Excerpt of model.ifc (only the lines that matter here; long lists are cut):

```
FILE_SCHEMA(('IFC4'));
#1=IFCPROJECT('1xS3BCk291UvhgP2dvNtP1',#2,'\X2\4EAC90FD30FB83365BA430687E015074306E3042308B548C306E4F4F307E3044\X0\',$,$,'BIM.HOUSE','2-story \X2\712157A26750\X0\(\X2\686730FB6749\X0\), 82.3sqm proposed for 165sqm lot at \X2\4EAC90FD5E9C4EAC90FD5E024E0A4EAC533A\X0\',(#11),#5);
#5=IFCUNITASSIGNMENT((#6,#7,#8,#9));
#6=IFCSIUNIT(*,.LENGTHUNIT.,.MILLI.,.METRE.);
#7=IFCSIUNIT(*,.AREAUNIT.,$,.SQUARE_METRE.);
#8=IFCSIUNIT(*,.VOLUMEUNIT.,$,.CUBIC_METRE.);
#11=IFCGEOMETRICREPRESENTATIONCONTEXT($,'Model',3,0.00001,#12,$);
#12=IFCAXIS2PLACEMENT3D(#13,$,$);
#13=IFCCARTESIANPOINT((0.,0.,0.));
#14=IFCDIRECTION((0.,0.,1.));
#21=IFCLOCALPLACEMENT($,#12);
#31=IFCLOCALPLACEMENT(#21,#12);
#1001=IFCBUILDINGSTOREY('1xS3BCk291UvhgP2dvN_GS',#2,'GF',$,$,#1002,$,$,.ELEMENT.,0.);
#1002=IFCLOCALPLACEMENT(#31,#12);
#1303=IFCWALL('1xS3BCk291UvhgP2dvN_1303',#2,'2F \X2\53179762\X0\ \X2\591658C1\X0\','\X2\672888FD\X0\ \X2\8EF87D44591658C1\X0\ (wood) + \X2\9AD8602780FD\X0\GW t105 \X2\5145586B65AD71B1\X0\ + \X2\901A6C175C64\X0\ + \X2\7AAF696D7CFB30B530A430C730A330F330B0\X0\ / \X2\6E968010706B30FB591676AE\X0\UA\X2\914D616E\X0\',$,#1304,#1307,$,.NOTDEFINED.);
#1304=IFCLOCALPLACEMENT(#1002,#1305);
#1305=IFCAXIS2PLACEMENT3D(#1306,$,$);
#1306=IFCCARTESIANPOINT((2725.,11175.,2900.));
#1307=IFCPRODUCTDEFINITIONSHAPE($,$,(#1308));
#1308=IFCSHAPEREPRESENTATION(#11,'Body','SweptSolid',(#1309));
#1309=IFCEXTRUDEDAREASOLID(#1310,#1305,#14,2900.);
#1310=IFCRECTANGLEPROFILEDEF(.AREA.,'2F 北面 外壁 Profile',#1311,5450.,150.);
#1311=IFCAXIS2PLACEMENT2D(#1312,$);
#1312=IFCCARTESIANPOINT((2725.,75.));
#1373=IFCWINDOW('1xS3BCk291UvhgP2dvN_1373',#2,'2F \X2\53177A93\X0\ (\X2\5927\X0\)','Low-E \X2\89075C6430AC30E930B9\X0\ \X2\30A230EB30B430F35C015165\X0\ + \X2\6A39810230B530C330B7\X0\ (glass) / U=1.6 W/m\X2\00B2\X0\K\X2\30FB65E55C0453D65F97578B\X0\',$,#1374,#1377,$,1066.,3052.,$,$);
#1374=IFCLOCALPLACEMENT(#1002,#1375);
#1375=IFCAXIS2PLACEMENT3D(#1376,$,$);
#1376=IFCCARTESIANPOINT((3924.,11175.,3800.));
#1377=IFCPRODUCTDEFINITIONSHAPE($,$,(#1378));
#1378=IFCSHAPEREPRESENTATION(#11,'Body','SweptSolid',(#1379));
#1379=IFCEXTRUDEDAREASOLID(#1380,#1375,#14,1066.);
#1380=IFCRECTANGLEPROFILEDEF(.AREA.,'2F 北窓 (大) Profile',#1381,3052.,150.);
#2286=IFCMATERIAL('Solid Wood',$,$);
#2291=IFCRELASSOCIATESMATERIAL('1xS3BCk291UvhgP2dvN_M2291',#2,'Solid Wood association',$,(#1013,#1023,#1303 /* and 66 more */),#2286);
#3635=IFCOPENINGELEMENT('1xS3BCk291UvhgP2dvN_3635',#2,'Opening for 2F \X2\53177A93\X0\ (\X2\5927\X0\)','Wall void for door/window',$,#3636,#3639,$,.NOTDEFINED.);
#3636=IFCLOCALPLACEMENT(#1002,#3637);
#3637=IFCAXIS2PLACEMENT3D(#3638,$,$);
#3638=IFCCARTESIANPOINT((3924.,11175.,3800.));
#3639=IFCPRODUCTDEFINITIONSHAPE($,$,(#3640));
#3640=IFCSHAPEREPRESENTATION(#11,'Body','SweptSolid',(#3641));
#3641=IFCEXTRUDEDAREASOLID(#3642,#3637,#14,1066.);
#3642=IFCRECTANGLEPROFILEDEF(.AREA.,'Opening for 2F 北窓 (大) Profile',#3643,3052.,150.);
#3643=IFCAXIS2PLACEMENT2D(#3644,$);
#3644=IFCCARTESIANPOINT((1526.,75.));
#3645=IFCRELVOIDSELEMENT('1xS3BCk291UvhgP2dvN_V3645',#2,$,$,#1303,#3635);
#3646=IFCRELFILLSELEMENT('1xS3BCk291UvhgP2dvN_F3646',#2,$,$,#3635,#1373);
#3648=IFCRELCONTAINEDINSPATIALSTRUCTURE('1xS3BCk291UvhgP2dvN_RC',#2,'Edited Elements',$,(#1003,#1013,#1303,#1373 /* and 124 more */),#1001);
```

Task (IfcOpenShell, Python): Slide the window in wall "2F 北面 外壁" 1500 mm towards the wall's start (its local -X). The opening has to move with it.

```python
import ifcopenshell
import ifcopenshell.api.geometry
import ifcopenshell.util.placement
import ifcopenshell.util.unit

model = ifcopenshell.open("model.ifc")
unit_scale = ifcopenshell.util.unit.calculate_unit_scale(model)

window = model.by_id(1373)
opening = window.FillsVoids[0].RelatingOpeningElement
wall = opening.VoidsElements[0].RelatingBuildingElement

wall_matrix = ifcopenshell.util.placement.get_local_placement(wall.ObjectPlacement)
shift = wall_matrix[:3, 0] * -1.5 / unit_scale
before = ifcopenshell.util.placement.get_local_placement(window.ObjectPlacement)[:3, 3].copy()

# The window is not placed relative to its opening, so move both.
for product in (opening, window):
    matrix = ifcopenshell.util.placement.get_local_placement(product.ObjectPlacement)
    matrix[:3, 3] += shift
    ifcopenshell.api.geometry.edit_object_placement(model, product=product, matrix=matrix, is_si=False)

after = ifcopenshell.util.placement.get_local_placement(window.ObjectPlacement)[:3, 3]
print("window moved by", (after - before).round(3) + 0.0)

model.write("model_rev.ifc")
```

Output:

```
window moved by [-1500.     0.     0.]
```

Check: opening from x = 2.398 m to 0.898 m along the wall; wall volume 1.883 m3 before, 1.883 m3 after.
